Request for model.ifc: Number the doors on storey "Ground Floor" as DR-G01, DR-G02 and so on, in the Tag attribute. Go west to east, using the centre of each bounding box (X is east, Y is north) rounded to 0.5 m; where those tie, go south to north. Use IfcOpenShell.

First a look at what the model holds.

```python
import ifcopenshell
import ifcopenshell.util.element
import ifcopenshell.util.placement

model = ifcopenshell.open("model.ifc")
print(model.schema)
storey = next(s for s in model.by_type("IfcBuildingStorey") if s.Name == "Ground Floor")
doors = [e for e in ifcopenshell.util.element.get_decomposition(storey) if e.is_a("IfcDoor")]
for e in sorted(doors, key=lambda e: e.id()):
    origin = ifcopenshell.util.placement.get_local_placement(e.ObjectPlacement)[:3, 3]
    print(e.id(), e.Tag, e.Name, origin.round(2) + 0.0, sep=" | ")
```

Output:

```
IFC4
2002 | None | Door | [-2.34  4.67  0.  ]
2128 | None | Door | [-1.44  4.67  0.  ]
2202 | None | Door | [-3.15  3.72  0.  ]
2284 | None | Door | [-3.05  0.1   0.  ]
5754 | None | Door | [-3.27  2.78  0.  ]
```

```python
import ifcopenshell
import ifcopenshell.geom
import ifcopenshell.util.element
import ifcopenshell.util.shape

model = ifcopenshell.open("model.ifc")
settings = ifcopenshell.geom.settings()
settings.set("use-world-coords", True)


def centre(element):
    shape = ifcopenshell.geom.create_shape(settings, element)
    return ifcopenshell.util.shape.get_bbox_centroid(shape.geometry)


storey = next(s for s in model.by_type("IfcBuildingStorey") if s.Name == "Ground Floor")
doors = [e for e in ifcopenshell.util.element.get_decomposition(storey) if e.is_a("IfcDoor")]

# Insertion points can sit at a corner or the storey origin, so sort by the geometry (in metres).
centres = {e: centre(e) for e in doors}
doors.sort(key=lambda e: (round(centres[e][0] / 0.5), centres[e][1]))

for i, e in enumerate(doors, start=1):
    number = f"DR-G{i:02d}"
    e.Tag = number
    print(e.id(), number)

model.write("model-out.ifc")
```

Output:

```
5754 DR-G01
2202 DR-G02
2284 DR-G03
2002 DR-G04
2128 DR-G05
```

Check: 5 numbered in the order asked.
